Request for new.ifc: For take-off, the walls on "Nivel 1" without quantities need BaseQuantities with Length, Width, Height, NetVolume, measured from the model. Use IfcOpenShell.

First a look at what the model holds.

```python
import ifcopenshell
import ifcopenshell.util.element
import ifcopenshell.util.unit

model = ifcopenshell.open("new.ifc")
print(model.schema)
for unit_type in ("LENGTHUNIT", "AREAUNIT", "VOLUMEUNIT"):
    print(unit_type, ifcopenshell.util.unit.calculate_unit_scale(model, unit_type))
storey = next(s for s in model.by_type("IfcBuildingStorey") if s.Name == "Nivel 1")
walls = [e for e in ifcopenshell.util.element.get_decomposition(storey) if e.is_a("IfcWall")]
for e in sorted(walls, key=lambda e: e.id()):
    print(e.id(), e.is_a(), e.Name, list(ifcopenshell.util.element.get_psets(e, qtos_only=True)), sep=" | ")
```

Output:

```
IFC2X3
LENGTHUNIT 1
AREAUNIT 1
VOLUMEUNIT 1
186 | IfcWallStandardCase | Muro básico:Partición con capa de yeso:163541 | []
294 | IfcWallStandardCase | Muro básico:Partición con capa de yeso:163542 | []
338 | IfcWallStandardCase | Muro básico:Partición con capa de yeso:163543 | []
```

```python
import ifcopenshell
import ifcopenshell.api.pset
import ifcopenshell.geom
import ifcopenshell.util.element
import ifcopenshell.util.shape
import ifcopenshell.util.unit

model = ifcopenshell.open("new.ifc")
unit_scale = ifcopenshell.util.unit.calculate_unit_scale(model)
volume_scale = ifcopenshell.util.unit.calculate_unit_scale(model, "VOLUMEUNIT")
settings = ifcopenshell.geom.settings()

storey = next(s for s in model.by_type("IfcBuildingStorey") if s.Name == "Nivel 1")
walls = [e for e in ifcopenshell.util.element.get_decomposition(storey) if e.is_a("IfcWall")]

for e in sorted(walls, key=lambda e: e.id()):
    if ifcopenshell.util.element.get_psets(e, qtos_only=True, should_inherit=False):
        continue
    # Geometry comes back in metres, in the element's own axes.
    shape = ifcopenshell.geom.create_shape(settings, e)
    values = {
        "Length": ifcopenshell.util.shape.get_x(shape.geometry) / unit_scale,
        "Width": ifcopenshell.util.shape.get_y(shape.geometry) / unit_scale,
        "Height": ifcopenshell.util.shape.get_z(shape.geometry) / unit_scale,
        "NetVolume": ifcopenshell.util.shape.get_volume(shape.geometry) / volume_scale,
    }
    qto = ifcopenshell.api.pset.add_qto(model, product=e, name="BaseQuantities")
    ifcopenshell.api.pset.edit_qto(model, qto=qto, properties=values)
    print(e.id(), {k: round(v, 3) for k, v in values.items()})

model.write("new_edited.ifc")
```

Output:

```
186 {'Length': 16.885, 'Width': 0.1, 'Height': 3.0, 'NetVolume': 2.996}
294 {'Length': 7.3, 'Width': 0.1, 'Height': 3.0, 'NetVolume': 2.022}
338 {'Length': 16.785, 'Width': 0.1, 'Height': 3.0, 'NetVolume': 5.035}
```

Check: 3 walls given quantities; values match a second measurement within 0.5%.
